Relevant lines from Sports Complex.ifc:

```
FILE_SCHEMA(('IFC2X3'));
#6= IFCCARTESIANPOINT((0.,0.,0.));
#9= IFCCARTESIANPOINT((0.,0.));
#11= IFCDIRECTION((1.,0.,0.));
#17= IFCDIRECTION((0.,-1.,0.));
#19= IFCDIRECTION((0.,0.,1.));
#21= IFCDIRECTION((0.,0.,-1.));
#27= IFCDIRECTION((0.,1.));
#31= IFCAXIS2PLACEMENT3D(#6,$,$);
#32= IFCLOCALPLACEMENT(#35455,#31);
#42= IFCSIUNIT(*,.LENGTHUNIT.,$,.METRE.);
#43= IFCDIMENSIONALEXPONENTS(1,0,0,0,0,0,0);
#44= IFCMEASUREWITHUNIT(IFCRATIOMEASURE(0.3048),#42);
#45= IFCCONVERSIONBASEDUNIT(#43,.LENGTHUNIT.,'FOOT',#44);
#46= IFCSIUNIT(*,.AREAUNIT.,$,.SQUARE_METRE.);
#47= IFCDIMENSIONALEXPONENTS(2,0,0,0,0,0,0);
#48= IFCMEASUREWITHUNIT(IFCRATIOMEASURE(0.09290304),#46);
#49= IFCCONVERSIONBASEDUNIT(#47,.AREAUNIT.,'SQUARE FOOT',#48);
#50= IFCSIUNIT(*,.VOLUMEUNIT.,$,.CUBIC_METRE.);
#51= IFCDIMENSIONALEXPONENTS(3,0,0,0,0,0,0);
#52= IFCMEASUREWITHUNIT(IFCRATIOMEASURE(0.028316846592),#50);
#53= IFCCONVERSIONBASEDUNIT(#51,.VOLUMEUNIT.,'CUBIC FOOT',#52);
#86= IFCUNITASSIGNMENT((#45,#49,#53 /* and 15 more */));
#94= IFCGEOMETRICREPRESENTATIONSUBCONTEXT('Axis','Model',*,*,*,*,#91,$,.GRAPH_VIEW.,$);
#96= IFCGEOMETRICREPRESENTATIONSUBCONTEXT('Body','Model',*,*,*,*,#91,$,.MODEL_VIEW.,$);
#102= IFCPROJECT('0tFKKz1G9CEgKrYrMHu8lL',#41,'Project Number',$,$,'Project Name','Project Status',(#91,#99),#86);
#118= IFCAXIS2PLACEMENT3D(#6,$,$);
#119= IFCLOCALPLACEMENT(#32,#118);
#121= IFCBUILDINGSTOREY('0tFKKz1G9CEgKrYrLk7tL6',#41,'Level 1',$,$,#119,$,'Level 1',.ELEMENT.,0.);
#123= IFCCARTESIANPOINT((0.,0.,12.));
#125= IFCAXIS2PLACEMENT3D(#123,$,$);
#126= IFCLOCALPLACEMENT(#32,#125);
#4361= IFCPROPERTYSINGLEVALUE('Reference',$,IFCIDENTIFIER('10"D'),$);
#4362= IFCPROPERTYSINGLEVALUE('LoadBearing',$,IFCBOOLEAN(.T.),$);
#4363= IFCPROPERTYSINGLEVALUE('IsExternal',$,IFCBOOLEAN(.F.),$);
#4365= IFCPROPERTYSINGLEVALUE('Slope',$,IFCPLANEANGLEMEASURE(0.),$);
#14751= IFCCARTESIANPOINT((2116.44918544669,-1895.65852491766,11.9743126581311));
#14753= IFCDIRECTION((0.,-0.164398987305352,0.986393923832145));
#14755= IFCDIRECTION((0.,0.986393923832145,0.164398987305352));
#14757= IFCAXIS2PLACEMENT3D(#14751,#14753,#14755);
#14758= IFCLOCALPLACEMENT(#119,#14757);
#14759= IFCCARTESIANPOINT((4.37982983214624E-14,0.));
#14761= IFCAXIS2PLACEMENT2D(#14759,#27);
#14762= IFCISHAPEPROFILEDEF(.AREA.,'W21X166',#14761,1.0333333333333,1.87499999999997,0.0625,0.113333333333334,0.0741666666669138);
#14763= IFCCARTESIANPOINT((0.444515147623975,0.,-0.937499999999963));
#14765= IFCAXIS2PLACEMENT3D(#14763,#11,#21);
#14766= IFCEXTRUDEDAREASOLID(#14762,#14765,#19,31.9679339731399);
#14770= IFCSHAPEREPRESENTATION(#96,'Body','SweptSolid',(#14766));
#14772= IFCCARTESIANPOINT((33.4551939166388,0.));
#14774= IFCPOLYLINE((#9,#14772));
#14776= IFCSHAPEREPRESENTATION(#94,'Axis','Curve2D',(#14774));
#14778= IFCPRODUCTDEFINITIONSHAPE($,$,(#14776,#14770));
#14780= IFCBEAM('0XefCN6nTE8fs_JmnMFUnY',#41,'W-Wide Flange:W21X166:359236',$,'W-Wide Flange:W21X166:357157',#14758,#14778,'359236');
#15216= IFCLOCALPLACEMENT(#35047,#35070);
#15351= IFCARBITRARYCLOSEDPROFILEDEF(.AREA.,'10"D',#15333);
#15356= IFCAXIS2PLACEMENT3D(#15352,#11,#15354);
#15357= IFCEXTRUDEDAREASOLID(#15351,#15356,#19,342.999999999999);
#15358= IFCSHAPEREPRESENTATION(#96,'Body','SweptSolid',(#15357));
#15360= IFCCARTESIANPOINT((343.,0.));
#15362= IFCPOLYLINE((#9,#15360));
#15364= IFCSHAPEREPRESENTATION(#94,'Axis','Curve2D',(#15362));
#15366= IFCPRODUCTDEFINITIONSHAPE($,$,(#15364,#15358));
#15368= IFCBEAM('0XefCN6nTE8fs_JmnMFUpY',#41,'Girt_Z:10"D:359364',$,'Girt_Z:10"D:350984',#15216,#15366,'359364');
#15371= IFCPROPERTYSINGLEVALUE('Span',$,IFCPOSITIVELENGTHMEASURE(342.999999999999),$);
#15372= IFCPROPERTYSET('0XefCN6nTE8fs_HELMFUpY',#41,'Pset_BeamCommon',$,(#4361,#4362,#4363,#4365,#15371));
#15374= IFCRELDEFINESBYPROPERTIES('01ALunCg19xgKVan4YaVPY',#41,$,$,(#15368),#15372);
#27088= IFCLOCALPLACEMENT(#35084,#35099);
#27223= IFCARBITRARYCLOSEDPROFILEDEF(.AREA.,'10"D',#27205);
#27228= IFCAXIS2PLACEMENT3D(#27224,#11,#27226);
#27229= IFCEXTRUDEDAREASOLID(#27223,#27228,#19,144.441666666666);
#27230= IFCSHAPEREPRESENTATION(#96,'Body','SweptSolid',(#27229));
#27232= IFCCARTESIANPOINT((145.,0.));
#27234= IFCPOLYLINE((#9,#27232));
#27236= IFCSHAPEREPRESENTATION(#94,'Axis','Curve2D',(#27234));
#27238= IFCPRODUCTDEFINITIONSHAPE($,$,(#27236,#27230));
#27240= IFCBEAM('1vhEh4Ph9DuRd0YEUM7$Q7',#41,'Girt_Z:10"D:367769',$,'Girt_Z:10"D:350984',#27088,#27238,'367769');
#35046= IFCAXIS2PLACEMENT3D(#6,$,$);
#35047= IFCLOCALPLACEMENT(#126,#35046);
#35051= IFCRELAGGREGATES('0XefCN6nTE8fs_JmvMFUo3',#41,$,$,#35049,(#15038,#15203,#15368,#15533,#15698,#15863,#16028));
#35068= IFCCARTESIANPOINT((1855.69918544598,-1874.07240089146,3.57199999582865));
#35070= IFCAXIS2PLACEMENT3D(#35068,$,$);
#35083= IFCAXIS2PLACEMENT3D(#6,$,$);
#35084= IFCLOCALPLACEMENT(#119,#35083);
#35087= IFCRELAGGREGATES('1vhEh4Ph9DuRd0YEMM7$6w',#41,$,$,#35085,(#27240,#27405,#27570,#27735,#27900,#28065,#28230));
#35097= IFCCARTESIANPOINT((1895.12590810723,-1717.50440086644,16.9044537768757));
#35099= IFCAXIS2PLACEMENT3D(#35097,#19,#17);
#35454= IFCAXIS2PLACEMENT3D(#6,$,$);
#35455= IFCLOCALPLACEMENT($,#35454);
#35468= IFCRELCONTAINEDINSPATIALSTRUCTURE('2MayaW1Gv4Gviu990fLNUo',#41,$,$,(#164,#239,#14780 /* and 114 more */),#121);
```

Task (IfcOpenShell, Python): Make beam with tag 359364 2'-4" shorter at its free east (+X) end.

```python
import numpy as np
import ifcopenshell
import ifcopenshell.api.pset
import ifcopenshell.util.element
import ifcopenshell.util.representation
import ifcopenshell.util.unit

model = ifcopenshell.open("Sports Complex.ifc")
unit_scale = ifcopenshell.util.unit.calculate_unit_scale(model)

member = model.by_guid("0XefCN6nTE8fs_JmnMFUpY")
change = -28 * 0.0254 / unit_scale

# The extrusion runs towards the end named, so only its depth changes.
body = ifcopenshell.util.representation.get_representation(member, "Model", "Body")
solid = body.Items[0]
old_length = solid.Depth
solid.Depth += change

# Move the axis end point with it.
axis = next(r for r in member.Representation.Representations if r.RepresentationIdentifier == "Axis").Items[0]
start, end = (np.array(p.Coordinates) for p in axis.Points)
end = end + (end - start) / np.linalg.norm(end - start) * change
point = model.createIfcCartesianPoint(end.tolist())
axis.Points = [axis.Points[0], point]

# Update the stored length and volume.
pset = model.by_id(ifcopenshell.util.element.get_pset(member, "Pset_BeamCommon", should_inherit=False)["id"])
ifcopenshell.api.pset.edit_pset(model, pset=pset, properties={
    "Span": model.create_entity("IfcPositiveLengthMeasure", solid.Depth),
})

print(f"length {old_length:g} -> {solid.Depth:g}")

model.write("Sports Complex_updated.ifc")
```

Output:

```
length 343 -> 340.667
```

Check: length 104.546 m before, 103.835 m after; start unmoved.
